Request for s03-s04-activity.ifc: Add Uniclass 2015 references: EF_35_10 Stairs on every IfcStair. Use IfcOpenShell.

First a look at what the model holds.

```python
import ifcopenshell

model = ifcopenshell.open("s03-s04-activity.ifc")
print(model.schema)
print("classifications:", [c.Name for c in model.by_type("IfcClassification")])
for ifc_class in ("IfcDoor", "IfcRoof", "IfcStair", "IfcWall", "IfcWindow"):
    print(ifc_class, len(model.by_type(ifc_class)))
```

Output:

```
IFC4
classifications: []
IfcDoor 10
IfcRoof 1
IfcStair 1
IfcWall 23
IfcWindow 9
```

```python
import ifcopenshell
import ifcopenshell.api.classification

model = ifcopenshell.open("s03-s04-activity.ifc")

system = ifcopenshell.api.classification.add_classification(model, classification="Uniclass 2015")

codes = {
    "IfcStair": ("EF_35_10", "Stairs"),
}
for ifc_class, (code, name) in codes.items():
    products = model.by_type(ifc_class)
    ifcopenshell.api.classification.add_reference(
        model, products=products, classification=system, identification=code, name=name
    )
    print(code, len(products))

model.write("s03-s04-activity-out.ifc")
```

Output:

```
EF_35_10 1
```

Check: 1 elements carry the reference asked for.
